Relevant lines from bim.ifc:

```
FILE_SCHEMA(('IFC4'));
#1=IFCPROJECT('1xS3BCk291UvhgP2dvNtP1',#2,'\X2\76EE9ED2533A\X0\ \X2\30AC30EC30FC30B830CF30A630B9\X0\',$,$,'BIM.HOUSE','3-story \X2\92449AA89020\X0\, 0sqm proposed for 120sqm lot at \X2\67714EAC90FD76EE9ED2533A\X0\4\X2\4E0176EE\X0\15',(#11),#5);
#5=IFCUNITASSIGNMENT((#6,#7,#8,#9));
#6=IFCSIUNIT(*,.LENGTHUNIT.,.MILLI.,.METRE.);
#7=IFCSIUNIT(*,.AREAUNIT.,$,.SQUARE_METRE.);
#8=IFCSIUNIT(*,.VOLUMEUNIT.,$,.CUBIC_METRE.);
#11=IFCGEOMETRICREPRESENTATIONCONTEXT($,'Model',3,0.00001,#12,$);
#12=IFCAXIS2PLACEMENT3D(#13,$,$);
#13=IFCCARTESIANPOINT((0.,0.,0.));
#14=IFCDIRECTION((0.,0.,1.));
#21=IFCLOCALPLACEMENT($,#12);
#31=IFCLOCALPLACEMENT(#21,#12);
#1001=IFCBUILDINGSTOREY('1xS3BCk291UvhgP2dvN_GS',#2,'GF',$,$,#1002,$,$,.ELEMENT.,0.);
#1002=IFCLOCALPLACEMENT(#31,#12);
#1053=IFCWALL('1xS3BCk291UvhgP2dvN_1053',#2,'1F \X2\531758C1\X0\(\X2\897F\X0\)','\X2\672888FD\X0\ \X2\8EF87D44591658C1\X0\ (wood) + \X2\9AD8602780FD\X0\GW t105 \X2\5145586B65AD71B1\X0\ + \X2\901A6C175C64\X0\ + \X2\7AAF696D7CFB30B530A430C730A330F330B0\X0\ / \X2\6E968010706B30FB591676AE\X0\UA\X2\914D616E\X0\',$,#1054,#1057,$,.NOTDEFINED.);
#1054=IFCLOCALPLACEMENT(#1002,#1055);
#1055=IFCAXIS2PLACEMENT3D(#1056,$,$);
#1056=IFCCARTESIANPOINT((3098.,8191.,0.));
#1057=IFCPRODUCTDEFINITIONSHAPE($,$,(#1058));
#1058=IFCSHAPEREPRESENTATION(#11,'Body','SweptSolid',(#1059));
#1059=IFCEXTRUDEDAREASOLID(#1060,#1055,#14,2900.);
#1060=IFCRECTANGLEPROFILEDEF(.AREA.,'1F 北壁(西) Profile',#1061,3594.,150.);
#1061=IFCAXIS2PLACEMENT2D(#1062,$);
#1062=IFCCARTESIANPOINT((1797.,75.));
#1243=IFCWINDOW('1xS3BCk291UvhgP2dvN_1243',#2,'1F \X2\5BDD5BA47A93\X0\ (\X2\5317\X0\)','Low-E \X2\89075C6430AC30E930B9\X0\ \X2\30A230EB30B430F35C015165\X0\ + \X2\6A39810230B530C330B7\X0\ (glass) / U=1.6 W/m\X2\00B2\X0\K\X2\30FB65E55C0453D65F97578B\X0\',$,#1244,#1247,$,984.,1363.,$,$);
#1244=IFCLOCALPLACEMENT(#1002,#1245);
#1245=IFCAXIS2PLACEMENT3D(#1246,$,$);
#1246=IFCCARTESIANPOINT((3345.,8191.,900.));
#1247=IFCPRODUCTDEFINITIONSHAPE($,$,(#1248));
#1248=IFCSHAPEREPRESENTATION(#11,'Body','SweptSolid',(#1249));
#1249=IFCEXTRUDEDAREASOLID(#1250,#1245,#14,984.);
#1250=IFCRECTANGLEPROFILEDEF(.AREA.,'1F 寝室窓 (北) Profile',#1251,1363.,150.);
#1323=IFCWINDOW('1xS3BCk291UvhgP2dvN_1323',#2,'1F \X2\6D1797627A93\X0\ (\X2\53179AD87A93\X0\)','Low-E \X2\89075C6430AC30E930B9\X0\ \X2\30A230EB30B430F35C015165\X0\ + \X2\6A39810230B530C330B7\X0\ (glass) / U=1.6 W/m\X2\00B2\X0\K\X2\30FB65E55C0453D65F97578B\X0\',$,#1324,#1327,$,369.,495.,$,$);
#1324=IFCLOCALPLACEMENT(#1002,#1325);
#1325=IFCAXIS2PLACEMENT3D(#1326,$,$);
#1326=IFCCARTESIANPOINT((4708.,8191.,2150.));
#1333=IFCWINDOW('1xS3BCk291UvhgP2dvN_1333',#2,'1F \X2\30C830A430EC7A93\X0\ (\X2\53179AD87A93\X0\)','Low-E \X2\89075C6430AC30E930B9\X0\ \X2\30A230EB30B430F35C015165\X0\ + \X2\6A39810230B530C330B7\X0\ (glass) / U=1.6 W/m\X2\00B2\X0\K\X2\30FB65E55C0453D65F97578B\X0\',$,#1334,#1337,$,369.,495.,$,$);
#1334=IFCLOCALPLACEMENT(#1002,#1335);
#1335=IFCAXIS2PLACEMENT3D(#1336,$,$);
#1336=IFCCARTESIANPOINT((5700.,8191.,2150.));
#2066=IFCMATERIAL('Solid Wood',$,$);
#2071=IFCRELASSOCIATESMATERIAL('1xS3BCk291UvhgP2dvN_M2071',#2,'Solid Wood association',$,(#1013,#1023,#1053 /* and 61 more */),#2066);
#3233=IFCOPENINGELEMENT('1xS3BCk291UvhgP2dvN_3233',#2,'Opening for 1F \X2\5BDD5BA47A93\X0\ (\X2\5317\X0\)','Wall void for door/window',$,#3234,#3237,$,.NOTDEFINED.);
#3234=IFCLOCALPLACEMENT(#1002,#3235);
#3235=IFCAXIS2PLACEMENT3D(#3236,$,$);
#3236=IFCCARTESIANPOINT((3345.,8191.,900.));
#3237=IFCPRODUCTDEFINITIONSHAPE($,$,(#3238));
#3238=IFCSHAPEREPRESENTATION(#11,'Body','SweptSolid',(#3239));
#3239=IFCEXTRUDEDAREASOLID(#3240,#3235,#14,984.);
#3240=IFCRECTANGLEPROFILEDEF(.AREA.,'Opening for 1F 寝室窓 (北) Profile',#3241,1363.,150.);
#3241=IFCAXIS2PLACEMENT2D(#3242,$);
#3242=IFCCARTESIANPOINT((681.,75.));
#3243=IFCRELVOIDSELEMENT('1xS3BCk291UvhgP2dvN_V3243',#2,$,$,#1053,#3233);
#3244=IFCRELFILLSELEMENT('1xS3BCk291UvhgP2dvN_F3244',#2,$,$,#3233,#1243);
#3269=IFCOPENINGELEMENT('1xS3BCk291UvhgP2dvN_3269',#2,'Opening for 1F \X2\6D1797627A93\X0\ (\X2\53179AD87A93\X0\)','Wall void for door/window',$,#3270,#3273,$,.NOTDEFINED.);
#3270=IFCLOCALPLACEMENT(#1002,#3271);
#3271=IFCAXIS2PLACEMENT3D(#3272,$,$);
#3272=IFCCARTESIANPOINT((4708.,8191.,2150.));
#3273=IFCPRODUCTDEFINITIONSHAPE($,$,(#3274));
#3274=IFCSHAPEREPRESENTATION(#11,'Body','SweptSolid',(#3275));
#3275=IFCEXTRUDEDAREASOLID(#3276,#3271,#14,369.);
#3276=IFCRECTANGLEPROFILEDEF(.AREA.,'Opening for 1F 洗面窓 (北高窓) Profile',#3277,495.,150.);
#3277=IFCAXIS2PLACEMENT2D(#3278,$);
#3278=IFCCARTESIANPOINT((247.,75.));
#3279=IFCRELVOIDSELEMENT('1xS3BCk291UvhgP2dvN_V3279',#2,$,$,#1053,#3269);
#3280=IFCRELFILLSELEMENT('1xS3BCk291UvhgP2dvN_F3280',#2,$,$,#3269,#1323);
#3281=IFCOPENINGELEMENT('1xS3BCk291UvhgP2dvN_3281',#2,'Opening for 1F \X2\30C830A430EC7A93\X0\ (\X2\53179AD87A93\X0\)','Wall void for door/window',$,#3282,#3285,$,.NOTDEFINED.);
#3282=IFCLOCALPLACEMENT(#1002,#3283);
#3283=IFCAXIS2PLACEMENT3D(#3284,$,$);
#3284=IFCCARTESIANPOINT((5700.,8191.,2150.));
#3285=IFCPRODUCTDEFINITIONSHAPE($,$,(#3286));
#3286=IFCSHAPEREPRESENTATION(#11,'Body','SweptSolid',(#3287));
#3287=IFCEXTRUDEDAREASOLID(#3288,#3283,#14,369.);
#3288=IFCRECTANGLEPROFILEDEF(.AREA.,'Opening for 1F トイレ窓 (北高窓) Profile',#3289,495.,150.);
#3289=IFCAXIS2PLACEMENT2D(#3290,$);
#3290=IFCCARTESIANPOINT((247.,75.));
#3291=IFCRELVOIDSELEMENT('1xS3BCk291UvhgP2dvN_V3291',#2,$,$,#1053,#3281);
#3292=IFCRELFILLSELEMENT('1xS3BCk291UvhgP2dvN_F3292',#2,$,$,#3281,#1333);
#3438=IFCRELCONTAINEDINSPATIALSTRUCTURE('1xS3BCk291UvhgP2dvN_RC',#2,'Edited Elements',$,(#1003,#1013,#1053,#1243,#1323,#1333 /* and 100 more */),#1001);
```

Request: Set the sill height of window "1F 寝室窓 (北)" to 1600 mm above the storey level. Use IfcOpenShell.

```python
import numpy as np
import ifcopenshell
import ifcopenshell.api.geometry
import ifcopenshell.geom
import ifcopenshell.util.element
import ifcopenshell.util.placement
import ifcopenshell.util.shape
import ifcopenshell.util.unit

model = ifcopenshell.open("bim.ifc")
unit_scale = ifcopenshell.util.unit.calculate_unit_scale(model)

window = model.by_guid("1xS3BCk291UvhgP2dvN_1243")
opening = window.FillsVoids[0].RelatingOpeningElement
storey = ifcopenshell.util.element.get_container(window, ifc_class="IfcBuildingStorey")
level = ifcopenshell.util.placement.get_local_placement(storey.ObjectPlacement)[2, 3]

# The opening's origin need not be at the sill, so measure its lowest point.
shape = ifcopenshell.geom.create_shape(ifcopenshell.geom.settings(), opening)
bottom = ifcopenshell.util.shape.get_shape_bottom_elevation(shape, shape.geometry) / unit_scale
dz = level + 1600.0 - bottom

shift = np.array([0.0, 0.0, dz])
# The window is not placed relative to its opening, so move both.
for product in (opening, window):
    matrix = ifcopenshell.util.placement.get_local_placement(product.ObjectPlacement)
    matrix[:3, 3] += shift
    ifcopenshell.api.geometry.edit_object_placement(model, product=product, matrix=matrix, is_si=False)

print(f"moved by {dz * unit_scale:+.3f} m")

model.write("bim-out.ifc")
```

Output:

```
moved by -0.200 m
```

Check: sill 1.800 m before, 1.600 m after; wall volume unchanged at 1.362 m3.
